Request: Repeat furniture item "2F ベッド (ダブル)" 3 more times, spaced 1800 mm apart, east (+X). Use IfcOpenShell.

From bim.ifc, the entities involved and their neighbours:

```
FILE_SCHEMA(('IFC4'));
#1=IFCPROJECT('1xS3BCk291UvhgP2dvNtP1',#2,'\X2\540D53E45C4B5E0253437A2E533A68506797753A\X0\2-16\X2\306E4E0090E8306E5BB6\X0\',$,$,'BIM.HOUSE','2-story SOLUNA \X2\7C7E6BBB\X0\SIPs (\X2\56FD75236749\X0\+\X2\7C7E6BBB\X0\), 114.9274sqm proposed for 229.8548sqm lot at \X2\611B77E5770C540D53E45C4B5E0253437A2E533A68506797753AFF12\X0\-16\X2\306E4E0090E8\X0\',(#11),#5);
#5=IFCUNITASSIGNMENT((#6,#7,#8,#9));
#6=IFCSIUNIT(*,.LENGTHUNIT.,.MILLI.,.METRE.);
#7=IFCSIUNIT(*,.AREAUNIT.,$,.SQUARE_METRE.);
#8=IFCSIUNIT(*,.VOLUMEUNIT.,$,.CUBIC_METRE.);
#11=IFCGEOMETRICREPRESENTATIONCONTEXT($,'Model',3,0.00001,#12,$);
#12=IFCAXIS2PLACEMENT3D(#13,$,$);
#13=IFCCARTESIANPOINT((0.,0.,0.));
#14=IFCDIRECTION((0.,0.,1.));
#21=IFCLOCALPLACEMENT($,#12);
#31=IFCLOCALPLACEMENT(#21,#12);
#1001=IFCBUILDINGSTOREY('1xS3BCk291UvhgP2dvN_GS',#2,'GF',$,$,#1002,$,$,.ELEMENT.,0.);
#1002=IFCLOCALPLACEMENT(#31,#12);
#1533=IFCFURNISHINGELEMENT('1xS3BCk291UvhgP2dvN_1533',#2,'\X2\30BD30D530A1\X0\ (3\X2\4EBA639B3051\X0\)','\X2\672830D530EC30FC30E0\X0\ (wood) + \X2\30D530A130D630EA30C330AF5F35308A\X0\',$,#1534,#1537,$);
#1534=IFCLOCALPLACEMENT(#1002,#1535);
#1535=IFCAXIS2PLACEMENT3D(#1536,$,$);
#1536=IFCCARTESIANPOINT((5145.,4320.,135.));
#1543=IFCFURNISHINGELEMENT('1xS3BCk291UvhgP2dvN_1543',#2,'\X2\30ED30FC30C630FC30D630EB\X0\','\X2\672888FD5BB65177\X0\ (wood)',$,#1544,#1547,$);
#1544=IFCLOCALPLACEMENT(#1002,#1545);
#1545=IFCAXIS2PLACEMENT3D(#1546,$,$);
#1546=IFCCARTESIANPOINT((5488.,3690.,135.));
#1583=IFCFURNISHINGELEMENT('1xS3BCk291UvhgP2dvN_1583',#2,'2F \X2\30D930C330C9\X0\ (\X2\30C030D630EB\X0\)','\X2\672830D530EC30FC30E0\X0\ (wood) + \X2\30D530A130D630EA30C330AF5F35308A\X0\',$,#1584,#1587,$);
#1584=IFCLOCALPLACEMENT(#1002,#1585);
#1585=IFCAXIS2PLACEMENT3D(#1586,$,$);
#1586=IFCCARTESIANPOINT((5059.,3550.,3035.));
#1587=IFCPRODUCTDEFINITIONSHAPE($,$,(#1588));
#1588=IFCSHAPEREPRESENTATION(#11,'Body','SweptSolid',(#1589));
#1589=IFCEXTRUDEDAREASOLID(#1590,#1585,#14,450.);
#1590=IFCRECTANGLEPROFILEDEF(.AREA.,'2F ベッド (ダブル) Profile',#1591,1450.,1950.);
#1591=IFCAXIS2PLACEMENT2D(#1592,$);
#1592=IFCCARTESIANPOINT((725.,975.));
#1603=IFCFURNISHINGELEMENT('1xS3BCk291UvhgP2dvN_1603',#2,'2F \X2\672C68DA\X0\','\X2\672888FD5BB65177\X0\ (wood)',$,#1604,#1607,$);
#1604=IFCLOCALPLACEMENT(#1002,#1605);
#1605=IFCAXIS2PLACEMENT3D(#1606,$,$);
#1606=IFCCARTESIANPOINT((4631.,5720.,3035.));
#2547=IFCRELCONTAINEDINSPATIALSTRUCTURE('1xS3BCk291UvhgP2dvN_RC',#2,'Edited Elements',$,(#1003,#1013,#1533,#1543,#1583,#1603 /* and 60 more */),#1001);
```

```python
import numpy as np
import ifcopenshell
import ifcopenshell.api.geometry
import ifcopenshell.api.root
import ifcopenshell.util.element
import ifcopenshell.util.placement

model = ifcopenshell.open("bim.ifc")


def reuse_history(source, copy):
    """copy_class also copies each property set's owner history, people and application; keep the originals."""
    for rel in copy.IsDefinedBy:
        if rel.is_a("IfcRelDefinesByProperties") and (history := rel.RelatingPropertyDefinition.OwnerHistory):
            rel.RelatingPropertyDefinition.OwnerHistory = source.OwnerHistory
            ifcopenshell.util.element.remove_deep2(model, history)


source = model.by_guid("1xS3BCk291UvhgP2dvN_1583")
base = ifcopenshell.util.placement.get_local_placement(source.ObjectPlacement)
step = np.array([1.0, 0.0, 0.0]) * 1800.0

for i in range(1, 4):
    copy = ifcopenshell.api.root.copy_class(model, product=source)
    copy.Representation = ifcopenshell.util.element.copy_deep(
        model, source.Representation, exclude=["IfcGeometricRepresentationContext", "IfcRepresentationMap"]
    )
    reuse_history(source, copy)
    matrix = base.copy()
    matrix[:3, 3] += i * step
    print("added at", matrix[:3, 3].round(3) + 0.0)
    ifcopenshell.api.geometry.edit_object_placement(model, product=copy, matrix=matrix, is_si=False)

model.write("bim_v2.ifc")
```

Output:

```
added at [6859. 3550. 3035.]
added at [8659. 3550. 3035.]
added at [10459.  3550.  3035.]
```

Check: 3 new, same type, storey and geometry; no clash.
